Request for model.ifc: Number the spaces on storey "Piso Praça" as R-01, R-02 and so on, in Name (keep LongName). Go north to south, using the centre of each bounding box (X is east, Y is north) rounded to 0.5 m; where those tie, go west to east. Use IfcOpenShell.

First a look at what the model holds.

```python
import ifcopenshell
import ifcopenshell.util.element
import ifcopenshell.util.placement

model = ifcopenshell.open("model.ifc")
print(model.schema)
storey = next(s for s in model.by_type("IfcBuildingStorey") if s.Name == "Piso Praça")
spaces = [e for e in ifcopenshell.util.element.get_decomposition(storey) if e.is_a("IfcSpace")]
for e in sorted(spaces, key=lambda e: e.id()):
    origin = ifcopenshell.util.placement.get_local_placement(e.ObjectPlacement)[:3, 3]
    print(e.id(), e.Name, e.LongName, origin.round(2) + 0.0, sep=" | ")
```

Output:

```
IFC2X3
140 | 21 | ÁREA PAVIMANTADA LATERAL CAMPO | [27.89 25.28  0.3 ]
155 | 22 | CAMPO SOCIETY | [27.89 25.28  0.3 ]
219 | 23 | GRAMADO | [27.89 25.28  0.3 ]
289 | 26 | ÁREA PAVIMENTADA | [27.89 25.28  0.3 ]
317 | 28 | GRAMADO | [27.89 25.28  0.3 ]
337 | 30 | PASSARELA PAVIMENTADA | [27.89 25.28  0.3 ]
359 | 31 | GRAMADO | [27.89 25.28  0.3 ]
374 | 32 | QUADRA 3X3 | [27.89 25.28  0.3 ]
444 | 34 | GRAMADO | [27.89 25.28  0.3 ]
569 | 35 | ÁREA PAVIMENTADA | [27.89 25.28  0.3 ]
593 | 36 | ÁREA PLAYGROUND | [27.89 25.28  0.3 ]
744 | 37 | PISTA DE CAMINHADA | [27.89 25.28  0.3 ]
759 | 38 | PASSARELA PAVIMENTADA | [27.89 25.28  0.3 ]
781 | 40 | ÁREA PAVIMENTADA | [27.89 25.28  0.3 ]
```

```python
import ifcopenshell
import ifcopenshell.geom
import ifcopenshell.util.element
import ifcopenshell.util.shape

model = ifcopenshell.open("model.ifc")
settings = ifcopenshell.geom.settings()
settings.set("use-world-coords", True)


def centre(element):
    shape = ifcopenshell.geom.create_shape(settings, element)
    return ifcopenshell.util.shape.get_bbox_centroid(shape.geometry)


storey = next(s for s in model.by_type("IfcBuildingStorey") if s.Name == "Piso Praça")
spaces = [e for e in ifcopenshell.util.element.get_decomposition(storey) if e.is_a("IfcSpace")]

# Insertion points can sit at a corner or the storey origin, so sort by the geometry (in metres).
centres = {e: centre(e) for e in spaces}
spaces.sort(key=lambda e: (-round(centres[e][1] / 0.5), centres[e][0]))

for i, e in enumerate(spaces, start=1):
    number = f"R-{i:02d}"
    e.Name = number
    print(e.id(), number)

model.write("model-out.ifc")
```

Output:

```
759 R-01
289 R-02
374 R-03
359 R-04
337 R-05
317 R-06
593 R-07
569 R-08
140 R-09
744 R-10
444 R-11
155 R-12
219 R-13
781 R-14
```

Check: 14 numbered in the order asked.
